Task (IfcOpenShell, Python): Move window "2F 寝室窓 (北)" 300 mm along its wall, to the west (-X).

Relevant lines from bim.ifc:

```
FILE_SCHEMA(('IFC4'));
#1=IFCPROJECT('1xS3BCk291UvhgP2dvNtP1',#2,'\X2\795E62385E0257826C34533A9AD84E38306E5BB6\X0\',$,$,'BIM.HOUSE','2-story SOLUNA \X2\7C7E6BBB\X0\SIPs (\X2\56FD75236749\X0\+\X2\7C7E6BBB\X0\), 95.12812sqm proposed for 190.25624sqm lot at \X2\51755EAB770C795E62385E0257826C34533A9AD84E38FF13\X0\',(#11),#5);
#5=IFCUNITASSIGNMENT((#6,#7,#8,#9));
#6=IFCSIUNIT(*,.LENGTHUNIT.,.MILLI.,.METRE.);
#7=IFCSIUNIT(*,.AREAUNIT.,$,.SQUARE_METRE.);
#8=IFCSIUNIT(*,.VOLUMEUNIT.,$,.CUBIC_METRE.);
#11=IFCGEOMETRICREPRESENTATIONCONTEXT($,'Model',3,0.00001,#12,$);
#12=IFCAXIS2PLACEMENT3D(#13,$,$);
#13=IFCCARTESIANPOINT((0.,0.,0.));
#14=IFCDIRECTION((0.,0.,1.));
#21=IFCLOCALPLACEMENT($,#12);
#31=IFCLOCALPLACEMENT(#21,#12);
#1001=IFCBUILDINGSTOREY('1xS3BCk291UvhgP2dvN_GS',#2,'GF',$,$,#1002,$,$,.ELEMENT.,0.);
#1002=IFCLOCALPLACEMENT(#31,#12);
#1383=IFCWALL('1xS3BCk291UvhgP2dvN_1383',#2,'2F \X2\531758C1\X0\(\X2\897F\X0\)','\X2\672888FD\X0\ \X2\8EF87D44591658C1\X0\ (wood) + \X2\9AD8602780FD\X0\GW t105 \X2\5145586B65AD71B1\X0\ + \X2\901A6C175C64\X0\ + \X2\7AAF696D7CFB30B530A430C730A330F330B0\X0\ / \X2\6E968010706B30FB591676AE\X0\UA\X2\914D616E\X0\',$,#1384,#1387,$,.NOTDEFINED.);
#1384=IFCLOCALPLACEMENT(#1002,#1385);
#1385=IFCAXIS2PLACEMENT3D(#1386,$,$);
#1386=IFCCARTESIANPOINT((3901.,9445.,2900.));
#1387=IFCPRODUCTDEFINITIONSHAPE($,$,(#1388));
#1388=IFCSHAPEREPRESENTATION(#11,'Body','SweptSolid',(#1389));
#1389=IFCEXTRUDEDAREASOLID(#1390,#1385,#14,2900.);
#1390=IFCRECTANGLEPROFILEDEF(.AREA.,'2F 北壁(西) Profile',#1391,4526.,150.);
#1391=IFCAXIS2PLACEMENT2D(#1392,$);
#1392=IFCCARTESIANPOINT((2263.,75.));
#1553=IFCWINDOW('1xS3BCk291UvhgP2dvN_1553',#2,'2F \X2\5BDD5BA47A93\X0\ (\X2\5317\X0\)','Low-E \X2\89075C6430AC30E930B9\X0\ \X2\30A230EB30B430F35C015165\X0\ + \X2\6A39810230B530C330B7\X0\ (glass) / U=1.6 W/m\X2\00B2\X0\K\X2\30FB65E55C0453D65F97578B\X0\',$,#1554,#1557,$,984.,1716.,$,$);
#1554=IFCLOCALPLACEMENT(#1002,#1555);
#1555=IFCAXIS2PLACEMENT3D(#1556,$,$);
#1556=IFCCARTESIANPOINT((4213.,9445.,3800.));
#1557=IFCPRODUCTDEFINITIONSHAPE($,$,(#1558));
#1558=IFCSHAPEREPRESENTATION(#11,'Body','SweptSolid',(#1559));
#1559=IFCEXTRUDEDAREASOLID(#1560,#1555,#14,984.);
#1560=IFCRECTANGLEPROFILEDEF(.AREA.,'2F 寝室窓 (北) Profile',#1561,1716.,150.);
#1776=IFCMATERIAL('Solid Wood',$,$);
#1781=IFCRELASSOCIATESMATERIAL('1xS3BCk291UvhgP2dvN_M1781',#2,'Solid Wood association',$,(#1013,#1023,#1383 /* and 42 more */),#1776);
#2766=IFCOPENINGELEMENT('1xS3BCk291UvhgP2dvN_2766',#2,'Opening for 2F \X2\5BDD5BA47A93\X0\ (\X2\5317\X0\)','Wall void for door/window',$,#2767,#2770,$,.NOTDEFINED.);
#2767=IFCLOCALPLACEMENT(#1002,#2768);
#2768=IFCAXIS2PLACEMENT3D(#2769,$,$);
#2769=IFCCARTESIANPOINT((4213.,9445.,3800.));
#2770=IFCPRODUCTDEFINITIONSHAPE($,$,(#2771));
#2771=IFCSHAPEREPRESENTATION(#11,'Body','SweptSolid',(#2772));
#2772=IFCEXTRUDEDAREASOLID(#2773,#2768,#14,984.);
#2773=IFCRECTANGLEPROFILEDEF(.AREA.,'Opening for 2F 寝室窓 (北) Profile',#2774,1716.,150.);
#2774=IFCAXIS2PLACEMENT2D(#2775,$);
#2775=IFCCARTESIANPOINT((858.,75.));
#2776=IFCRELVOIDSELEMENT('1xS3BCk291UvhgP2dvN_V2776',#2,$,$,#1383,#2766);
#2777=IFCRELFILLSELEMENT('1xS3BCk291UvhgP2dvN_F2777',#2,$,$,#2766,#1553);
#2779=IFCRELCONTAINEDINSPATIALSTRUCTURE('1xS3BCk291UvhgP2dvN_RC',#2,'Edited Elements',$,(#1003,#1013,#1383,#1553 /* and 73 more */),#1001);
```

```python
import ifcopenshell
import ifcopenshell.api.geometry
import ifcopenshell.util.placement
import ifcopenshell.util.unit

model = ifcopenshell.open("bim.ifc")
unit_scale = ifcopenshell.util.unit.calculate_unit_scale(model)

window = model.by_guid("1xS3BCk291UvhgP2dvN_1553")
opening = window.FillsVoids[0].RelatingOpeningElement
wall = opening.VoidsElements[0].RelatingBuildingElement

wall_matrix = ifcopenshell.util.placement.get_local_placement(wall.ObjectPlacement)
shift = wall_matrix[:3, 0] * -0.3 / unit_scale
before = ifcopenshell.util.placement.get_local_placement(window.ObjectPlacement)[:3, 3].copy()

# The window is not placed relative to its opening, so move both.
for product in (opening, window):
    matrix = ifcopenshell.util.placement.get_local_placement(product.ObjectPlacement)
    matrix[:3, 3] += shift
    ifcopenshell.api.geometry.edit_object_placement(model, product=product, matrix=matrix, is_si=False)

after = ifcopenshell.util.placement.get_local_placement(window.ObjectPlacement)[:3, 3]
print("window moved by", (after - before).round(3) + 0.0)

model.write("bim_edited.ifc")
```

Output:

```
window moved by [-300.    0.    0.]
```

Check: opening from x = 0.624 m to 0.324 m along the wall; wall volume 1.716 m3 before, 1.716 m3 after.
